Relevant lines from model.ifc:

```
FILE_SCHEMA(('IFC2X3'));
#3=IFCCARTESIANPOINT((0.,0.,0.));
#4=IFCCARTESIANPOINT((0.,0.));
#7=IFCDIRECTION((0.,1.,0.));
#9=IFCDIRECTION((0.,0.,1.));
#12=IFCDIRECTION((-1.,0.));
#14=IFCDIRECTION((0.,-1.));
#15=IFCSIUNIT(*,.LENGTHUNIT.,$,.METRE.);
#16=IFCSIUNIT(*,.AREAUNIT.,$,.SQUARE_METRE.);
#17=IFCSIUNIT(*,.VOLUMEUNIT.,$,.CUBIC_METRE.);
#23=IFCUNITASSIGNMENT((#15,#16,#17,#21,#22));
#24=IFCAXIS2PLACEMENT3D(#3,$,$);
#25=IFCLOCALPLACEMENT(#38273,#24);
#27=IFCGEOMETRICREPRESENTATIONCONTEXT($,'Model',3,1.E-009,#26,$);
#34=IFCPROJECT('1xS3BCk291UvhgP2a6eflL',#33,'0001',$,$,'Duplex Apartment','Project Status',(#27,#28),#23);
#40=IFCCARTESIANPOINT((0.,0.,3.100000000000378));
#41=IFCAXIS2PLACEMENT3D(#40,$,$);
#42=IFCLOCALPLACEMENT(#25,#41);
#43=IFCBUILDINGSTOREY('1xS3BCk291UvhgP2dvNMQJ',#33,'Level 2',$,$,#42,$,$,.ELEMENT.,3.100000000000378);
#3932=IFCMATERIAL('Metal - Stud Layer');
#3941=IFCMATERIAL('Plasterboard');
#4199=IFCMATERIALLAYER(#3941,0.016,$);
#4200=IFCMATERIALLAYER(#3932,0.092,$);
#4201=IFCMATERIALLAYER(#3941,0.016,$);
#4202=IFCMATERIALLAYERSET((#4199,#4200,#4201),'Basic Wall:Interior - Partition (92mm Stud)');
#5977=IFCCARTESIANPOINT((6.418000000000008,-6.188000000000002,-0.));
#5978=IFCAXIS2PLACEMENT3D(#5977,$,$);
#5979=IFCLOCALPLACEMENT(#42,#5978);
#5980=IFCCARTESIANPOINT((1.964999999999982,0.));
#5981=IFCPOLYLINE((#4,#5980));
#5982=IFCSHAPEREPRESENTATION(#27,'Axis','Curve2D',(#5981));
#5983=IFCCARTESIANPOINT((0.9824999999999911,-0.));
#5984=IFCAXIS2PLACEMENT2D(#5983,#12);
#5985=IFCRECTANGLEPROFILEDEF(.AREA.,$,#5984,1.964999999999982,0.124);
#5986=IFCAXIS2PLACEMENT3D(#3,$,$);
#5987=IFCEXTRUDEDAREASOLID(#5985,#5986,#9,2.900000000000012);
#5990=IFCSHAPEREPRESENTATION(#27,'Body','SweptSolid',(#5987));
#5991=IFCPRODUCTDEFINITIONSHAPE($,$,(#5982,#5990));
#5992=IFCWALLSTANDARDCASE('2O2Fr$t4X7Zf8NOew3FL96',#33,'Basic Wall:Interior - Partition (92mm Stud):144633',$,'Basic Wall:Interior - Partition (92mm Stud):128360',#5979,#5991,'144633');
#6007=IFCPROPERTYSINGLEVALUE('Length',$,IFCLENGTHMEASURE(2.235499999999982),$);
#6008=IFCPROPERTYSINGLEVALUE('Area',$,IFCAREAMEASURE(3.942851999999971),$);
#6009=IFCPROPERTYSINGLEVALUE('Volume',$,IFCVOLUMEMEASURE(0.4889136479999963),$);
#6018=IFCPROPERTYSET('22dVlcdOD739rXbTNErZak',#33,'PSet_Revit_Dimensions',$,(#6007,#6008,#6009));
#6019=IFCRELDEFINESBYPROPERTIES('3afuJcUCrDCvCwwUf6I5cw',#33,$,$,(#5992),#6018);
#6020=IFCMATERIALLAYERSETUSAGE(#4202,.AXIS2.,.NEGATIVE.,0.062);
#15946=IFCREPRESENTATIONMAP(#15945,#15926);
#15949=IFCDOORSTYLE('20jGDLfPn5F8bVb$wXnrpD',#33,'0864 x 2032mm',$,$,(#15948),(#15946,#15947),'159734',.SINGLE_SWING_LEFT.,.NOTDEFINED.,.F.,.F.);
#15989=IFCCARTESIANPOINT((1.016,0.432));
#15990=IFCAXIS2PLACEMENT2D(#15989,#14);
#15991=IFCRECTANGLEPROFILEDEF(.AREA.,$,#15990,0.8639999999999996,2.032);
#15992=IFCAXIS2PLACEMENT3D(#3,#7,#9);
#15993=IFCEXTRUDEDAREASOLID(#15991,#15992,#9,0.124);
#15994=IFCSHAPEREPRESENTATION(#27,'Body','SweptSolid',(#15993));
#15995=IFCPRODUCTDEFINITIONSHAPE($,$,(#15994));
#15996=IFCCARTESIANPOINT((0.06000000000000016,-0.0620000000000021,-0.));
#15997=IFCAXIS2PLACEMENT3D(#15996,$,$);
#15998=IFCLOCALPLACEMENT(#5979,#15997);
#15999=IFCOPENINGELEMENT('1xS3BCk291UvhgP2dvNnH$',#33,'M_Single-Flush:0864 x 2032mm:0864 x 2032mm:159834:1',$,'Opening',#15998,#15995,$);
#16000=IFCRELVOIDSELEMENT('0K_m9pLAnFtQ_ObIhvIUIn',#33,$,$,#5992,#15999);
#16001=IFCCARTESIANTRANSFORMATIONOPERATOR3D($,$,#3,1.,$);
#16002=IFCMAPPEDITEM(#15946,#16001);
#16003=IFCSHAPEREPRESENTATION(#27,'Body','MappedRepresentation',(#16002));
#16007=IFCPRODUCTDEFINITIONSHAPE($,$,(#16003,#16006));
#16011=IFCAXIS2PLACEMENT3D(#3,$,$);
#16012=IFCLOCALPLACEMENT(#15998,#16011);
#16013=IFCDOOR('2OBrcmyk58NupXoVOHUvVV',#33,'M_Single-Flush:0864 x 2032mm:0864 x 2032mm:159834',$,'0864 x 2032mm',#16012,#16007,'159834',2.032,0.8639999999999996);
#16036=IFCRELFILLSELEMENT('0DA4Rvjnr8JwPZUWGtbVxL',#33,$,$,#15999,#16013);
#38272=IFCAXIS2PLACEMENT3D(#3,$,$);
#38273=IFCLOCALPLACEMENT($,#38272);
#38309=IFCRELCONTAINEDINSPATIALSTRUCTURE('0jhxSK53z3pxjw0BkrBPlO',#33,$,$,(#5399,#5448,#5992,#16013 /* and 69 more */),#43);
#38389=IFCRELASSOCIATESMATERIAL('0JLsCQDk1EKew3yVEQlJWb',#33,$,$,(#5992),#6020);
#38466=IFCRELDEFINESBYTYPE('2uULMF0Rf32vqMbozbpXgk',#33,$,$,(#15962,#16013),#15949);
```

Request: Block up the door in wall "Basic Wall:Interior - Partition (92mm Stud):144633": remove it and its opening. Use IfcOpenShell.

```python
import ifcopenshell
import ifcopenshell.api.feature
import ifcopenshell.api.pset
import ifcopenshell.api.root
import ifcopenshell.geom
import ifcopenshell.util.element
import ifcopenshell.util.shape
import ifcopenshell.util.unit

model = ifcopenshell.open("model.ifc")
area_scale = ifcopenshell.util.unit.calculate_unit_scale(model, "AREAUNIT")
volume_scale = ifcopenshell.util.unit.calculate_unit_scale(model, "VOLUMEUNIT")
settings = ifcopenshell.geom.settings()


def volume(element):
    """Net volume in cubic metres, openings subtracted."""
    shape = ifcopenshell.geom.create_shape(settings, element)
    return ifcopenshell.util.shape.get_volume(shape.geometry)


door = model.by_id(16013)
opening = door.FillsVoids[0].RelatingOpeningElement
wall = opening.VoidsElements[0].RelatingBuildingElement
before = volume(wall)

ifcopenshell.api.root.remove_product(model, product=door)
ifcopenshell.api.feature.remove_feature(model, feature=opening)

after = volume(wall)
thickness = 0.124  # wall thickness in metres

# Update the wall's stored quantities.
pset = model.by_id(ifcopenshell.util.element.get_pset(wall, "PSet_Revit_Dimensions", should_inherit=False)["id"])
ifcopenshell.api.pset.edit_pset(model, pset=pset, properties={
    "Area": model.create_entity("IfcAreaMeasure", after / thickness / area_scale),
    "Volume": model.create_entity("IfcVolumeMeasure", after / volume_scale),
})

print(f"wall volume {before:.3f} -> {after:.3f} m3")

model.write("model_rev.ifc")
```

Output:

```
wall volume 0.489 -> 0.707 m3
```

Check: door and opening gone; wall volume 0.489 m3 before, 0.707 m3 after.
